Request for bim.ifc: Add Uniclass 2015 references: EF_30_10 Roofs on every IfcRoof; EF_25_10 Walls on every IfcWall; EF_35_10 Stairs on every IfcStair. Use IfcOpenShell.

First a look at what the model holds.

```python
import ifcopenshell

model = ifcopenshell.open("bim.ifc")
print(model.schema)
print("classifications:", [c.Name for c in model.by_type("IfcClassification")])
for ifc_class in ("IfcDoor", "IfcRoof", "IfcStair", "IfcWall", "IfcWindow"):
    print(ifc_class, len(model.by_type(ifc_class)))
```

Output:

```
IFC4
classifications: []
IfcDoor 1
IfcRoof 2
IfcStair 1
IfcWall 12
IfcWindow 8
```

```python
import ifcopenshell
import ifcopenshell.api.classification

model = ifcopenshell.open("bim.ifc")

system = ifcopenshell.api.classification.add_classification(model, classification="Uniclass 2015")

codes = {
    "IfcRoof": ("EF_30_10", "Roofs"),
    "IfcWall": ("EF_25_10", "Walls"),
    "IfcStair": ("EF_35_10", "Stairs"),
}
for ifc_class, (code, name) in codes.items():
    products = model.by_type(ifc_class)
    ifcopenshell.api.classification.add_reference(
        model, products=products, classification=system, identification=code, name=name
    )
    print(code, len(products))

model.write("bim_v2.ifc")
```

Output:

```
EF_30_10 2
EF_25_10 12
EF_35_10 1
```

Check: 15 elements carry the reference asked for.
